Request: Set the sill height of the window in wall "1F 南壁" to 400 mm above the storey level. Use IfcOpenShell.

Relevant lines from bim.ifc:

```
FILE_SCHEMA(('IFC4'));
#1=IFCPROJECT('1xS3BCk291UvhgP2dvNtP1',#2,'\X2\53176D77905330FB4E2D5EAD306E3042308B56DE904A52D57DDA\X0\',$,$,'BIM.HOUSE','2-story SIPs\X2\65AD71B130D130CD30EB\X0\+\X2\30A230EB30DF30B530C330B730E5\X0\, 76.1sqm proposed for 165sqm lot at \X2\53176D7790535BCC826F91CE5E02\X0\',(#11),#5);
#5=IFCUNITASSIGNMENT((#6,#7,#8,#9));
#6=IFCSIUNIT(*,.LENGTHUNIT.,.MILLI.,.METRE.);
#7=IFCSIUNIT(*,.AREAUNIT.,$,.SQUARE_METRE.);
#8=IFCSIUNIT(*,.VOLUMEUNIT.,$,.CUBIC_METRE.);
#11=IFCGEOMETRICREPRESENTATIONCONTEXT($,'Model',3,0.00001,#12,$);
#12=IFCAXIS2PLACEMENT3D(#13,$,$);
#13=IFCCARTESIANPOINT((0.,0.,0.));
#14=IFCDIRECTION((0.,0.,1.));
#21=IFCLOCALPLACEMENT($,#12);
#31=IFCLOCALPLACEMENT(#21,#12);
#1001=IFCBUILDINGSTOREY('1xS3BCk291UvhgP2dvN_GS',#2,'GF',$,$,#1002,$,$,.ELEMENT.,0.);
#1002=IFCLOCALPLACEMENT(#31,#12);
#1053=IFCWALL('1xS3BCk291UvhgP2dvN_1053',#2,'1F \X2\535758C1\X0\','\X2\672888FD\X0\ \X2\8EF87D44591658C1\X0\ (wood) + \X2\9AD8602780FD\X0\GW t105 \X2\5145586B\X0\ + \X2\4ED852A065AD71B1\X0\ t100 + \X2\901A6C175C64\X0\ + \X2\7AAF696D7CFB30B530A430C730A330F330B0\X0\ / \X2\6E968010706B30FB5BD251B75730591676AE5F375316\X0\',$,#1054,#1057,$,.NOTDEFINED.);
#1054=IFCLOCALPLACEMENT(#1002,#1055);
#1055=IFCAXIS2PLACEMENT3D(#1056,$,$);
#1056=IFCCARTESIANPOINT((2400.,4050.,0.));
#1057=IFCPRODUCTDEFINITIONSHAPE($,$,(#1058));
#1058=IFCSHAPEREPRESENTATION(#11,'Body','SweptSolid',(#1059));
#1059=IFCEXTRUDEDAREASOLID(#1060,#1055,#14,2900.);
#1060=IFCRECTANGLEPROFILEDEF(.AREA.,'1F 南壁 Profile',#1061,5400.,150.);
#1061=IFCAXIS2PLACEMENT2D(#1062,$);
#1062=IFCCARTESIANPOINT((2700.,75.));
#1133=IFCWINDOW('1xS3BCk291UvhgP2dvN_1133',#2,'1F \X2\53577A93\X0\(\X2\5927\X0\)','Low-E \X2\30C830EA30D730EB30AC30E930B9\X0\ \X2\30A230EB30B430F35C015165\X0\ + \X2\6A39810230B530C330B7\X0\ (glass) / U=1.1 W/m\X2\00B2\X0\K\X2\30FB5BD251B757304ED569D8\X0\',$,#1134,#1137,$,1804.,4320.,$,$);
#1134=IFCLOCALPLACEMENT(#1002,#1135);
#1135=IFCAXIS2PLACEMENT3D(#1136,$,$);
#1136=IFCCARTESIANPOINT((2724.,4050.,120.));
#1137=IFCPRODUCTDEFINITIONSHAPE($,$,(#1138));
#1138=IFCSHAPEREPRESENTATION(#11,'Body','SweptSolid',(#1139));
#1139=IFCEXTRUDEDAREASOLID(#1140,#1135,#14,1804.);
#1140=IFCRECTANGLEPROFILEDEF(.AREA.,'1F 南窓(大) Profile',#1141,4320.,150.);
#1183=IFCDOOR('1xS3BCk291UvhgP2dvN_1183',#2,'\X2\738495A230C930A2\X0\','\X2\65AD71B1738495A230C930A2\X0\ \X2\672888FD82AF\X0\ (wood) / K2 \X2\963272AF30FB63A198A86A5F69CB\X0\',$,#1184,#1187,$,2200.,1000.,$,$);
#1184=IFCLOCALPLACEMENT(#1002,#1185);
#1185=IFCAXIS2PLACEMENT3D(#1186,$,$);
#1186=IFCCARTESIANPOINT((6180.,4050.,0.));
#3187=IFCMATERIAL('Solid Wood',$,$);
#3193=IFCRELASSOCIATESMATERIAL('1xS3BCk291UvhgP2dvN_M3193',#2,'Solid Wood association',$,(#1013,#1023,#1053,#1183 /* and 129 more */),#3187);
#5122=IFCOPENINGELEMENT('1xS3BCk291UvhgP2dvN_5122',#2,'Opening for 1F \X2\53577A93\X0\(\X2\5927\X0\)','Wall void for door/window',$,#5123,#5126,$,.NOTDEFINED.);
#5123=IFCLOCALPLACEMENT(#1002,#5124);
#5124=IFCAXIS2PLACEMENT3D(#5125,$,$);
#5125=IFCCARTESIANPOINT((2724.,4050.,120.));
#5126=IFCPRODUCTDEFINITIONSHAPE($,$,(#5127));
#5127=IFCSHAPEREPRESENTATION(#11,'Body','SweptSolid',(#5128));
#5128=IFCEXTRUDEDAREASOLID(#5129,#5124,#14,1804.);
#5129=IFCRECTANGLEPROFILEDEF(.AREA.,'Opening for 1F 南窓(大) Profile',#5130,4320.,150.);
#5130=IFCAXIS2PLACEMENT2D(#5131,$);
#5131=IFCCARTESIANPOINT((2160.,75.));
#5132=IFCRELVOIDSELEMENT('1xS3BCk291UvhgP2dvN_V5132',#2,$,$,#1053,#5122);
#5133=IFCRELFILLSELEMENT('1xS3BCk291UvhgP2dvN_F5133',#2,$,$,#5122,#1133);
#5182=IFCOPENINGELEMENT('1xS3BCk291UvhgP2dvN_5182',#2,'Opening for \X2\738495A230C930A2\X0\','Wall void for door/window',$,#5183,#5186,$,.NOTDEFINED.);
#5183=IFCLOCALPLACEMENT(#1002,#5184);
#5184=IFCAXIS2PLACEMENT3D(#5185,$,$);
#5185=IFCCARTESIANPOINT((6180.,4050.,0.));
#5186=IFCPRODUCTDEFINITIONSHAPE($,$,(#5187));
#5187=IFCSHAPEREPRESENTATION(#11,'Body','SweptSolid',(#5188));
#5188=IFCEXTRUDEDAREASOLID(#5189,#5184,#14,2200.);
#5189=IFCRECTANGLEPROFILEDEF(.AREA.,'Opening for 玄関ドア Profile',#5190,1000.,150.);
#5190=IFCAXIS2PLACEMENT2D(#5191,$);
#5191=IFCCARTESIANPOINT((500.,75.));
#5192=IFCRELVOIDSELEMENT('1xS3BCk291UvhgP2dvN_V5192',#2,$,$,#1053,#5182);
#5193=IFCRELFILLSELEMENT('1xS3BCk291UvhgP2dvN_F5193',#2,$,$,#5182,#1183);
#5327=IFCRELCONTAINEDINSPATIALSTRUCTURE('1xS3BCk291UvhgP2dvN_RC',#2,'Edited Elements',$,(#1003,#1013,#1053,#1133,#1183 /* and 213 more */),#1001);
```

```python
import numpy as np
import ifcopenshell
import ifcopenshell.api.geometry
import ifcopenshell.geom
import ifcopenshell.util.element
import ifcopenshell.util.placement
import ifcopenshell.util.shape
import ifcopenshell.util.unit

model = ifcopenshell.open("bim.ifc")
unit_scale = ifcopenshell.util.unit.calculate_unit_scale(model)

window = model.by_id(1133)
opening = window.FillsVoids[0].RelatingOpeningElement
storey = ifcopenshell.util.element.get_container(window, ifc_class="IfcBuildingStorey")
level = ifcopenshell.util.placement.get_local_placement(storey.ObjectPlacement)[2, 3]

# The opening's origin need not be at the sill, so measure its lowest point.
shape = ifcopenshell.geom.create_shape(ifcopenshell.geom.settings(), opening)
bottom = ifcopenshell.util.shape.get_shape_bottom_elevation(shape, shape.geometry) / unit_scale
dz = level + 0.4 / unit_scale - bottom

shift = np.array([0.0, 0.0, dz])
# The window is not placed relative to its opening, so move both.
for product in (opening, window):
    matrix = ifcopenshell.util.placement.get_local_placement(product.ObjectPlacement)
    matrix[:3, 3] += shift
    ifcopenshell.api.geometry.edit_object_placement(model, product=product, matrix=matrix, is_si=False)

print(f"moved by {dz * unit_scale:+.3f} m")

model.write("bim_rev.ifc")
```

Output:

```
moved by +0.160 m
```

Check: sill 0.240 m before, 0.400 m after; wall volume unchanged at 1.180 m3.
